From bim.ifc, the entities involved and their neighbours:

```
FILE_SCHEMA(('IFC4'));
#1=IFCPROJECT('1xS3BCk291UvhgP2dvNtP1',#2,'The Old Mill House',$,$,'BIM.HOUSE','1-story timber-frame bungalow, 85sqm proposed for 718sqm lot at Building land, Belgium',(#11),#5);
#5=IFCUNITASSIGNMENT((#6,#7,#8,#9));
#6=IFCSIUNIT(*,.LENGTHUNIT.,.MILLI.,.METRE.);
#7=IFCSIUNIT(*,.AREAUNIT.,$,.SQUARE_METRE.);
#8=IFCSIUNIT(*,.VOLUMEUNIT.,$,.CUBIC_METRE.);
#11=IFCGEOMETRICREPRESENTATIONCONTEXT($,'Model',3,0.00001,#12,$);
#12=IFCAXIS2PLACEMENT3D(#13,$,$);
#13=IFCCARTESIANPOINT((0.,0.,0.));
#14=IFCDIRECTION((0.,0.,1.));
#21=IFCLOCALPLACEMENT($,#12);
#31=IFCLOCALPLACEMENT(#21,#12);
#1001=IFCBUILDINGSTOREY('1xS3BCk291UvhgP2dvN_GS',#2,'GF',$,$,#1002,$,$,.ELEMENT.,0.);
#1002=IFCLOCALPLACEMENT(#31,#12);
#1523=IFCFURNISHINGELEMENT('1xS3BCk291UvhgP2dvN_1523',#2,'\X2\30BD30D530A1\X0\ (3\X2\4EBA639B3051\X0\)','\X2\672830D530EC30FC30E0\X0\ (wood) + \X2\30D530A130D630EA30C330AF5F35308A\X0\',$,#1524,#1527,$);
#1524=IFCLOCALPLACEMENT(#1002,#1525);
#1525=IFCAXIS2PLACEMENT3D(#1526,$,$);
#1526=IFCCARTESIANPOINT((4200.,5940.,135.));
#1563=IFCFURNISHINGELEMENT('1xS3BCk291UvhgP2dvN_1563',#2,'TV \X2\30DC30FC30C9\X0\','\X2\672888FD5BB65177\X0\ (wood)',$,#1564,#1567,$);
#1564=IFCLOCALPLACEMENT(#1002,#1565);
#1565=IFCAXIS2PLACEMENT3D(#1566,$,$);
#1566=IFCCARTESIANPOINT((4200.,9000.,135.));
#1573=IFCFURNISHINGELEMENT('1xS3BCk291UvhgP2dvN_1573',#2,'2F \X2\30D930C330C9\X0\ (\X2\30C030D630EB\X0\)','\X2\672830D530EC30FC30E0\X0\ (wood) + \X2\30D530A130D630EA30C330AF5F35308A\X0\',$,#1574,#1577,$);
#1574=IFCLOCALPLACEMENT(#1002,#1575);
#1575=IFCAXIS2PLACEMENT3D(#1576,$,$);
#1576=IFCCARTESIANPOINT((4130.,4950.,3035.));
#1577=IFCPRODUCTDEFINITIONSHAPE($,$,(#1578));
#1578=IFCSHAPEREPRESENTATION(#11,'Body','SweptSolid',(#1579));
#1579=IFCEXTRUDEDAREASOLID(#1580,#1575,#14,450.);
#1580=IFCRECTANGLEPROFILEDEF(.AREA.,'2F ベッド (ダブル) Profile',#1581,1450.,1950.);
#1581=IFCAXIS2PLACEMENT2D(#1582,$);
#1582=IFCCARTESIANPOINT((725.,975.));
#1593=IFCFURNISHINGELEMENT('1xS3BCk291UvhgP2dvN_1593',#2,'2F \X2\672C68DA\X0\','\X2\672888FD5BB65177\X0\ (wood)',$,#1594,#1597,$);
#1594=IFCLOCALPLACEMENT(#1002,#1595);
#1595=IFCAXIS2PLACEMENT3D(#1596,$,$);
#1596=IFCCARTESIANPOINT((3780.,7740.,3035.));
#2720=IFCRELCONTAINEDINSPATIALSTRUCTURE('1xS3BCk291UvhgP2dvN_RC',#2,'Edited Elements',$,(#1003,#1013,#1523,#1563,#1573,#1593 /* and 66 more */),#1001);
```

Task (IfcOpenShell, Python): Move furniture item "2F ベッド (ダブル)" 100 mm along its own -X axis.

```python
import ifcopenshell
import ifcopenshell.api.geometry
import ifcopenshell.util.placement

model = ifcopenshell.open("bim.ifc")

item = model.by_guid("1xS3BCk291UvhgP2dvN_1573")
matrix = ifcopenshell.util.placement.get_local_placement(item.ObjectPlacement)
matrix[:3, 3] -= matrix[:3, 0] * 100.0
ifcopenshell.api.geometry.edit_object_placement(model, product=item, matrix=matrix, is_si=False)

print(ifcopenshell.util.placement.get_local_placement(item.ObjectPlacement).round(3) + 0.0)

model.write("bim-out.ifc")
```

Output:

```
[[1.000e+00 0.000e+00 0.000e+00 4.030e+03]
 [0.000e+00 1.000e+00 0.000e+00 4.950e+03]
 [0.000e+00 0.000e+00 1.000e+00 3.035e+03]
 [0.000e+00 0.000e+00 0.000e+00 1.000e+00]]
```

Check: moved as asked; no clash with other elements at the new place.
